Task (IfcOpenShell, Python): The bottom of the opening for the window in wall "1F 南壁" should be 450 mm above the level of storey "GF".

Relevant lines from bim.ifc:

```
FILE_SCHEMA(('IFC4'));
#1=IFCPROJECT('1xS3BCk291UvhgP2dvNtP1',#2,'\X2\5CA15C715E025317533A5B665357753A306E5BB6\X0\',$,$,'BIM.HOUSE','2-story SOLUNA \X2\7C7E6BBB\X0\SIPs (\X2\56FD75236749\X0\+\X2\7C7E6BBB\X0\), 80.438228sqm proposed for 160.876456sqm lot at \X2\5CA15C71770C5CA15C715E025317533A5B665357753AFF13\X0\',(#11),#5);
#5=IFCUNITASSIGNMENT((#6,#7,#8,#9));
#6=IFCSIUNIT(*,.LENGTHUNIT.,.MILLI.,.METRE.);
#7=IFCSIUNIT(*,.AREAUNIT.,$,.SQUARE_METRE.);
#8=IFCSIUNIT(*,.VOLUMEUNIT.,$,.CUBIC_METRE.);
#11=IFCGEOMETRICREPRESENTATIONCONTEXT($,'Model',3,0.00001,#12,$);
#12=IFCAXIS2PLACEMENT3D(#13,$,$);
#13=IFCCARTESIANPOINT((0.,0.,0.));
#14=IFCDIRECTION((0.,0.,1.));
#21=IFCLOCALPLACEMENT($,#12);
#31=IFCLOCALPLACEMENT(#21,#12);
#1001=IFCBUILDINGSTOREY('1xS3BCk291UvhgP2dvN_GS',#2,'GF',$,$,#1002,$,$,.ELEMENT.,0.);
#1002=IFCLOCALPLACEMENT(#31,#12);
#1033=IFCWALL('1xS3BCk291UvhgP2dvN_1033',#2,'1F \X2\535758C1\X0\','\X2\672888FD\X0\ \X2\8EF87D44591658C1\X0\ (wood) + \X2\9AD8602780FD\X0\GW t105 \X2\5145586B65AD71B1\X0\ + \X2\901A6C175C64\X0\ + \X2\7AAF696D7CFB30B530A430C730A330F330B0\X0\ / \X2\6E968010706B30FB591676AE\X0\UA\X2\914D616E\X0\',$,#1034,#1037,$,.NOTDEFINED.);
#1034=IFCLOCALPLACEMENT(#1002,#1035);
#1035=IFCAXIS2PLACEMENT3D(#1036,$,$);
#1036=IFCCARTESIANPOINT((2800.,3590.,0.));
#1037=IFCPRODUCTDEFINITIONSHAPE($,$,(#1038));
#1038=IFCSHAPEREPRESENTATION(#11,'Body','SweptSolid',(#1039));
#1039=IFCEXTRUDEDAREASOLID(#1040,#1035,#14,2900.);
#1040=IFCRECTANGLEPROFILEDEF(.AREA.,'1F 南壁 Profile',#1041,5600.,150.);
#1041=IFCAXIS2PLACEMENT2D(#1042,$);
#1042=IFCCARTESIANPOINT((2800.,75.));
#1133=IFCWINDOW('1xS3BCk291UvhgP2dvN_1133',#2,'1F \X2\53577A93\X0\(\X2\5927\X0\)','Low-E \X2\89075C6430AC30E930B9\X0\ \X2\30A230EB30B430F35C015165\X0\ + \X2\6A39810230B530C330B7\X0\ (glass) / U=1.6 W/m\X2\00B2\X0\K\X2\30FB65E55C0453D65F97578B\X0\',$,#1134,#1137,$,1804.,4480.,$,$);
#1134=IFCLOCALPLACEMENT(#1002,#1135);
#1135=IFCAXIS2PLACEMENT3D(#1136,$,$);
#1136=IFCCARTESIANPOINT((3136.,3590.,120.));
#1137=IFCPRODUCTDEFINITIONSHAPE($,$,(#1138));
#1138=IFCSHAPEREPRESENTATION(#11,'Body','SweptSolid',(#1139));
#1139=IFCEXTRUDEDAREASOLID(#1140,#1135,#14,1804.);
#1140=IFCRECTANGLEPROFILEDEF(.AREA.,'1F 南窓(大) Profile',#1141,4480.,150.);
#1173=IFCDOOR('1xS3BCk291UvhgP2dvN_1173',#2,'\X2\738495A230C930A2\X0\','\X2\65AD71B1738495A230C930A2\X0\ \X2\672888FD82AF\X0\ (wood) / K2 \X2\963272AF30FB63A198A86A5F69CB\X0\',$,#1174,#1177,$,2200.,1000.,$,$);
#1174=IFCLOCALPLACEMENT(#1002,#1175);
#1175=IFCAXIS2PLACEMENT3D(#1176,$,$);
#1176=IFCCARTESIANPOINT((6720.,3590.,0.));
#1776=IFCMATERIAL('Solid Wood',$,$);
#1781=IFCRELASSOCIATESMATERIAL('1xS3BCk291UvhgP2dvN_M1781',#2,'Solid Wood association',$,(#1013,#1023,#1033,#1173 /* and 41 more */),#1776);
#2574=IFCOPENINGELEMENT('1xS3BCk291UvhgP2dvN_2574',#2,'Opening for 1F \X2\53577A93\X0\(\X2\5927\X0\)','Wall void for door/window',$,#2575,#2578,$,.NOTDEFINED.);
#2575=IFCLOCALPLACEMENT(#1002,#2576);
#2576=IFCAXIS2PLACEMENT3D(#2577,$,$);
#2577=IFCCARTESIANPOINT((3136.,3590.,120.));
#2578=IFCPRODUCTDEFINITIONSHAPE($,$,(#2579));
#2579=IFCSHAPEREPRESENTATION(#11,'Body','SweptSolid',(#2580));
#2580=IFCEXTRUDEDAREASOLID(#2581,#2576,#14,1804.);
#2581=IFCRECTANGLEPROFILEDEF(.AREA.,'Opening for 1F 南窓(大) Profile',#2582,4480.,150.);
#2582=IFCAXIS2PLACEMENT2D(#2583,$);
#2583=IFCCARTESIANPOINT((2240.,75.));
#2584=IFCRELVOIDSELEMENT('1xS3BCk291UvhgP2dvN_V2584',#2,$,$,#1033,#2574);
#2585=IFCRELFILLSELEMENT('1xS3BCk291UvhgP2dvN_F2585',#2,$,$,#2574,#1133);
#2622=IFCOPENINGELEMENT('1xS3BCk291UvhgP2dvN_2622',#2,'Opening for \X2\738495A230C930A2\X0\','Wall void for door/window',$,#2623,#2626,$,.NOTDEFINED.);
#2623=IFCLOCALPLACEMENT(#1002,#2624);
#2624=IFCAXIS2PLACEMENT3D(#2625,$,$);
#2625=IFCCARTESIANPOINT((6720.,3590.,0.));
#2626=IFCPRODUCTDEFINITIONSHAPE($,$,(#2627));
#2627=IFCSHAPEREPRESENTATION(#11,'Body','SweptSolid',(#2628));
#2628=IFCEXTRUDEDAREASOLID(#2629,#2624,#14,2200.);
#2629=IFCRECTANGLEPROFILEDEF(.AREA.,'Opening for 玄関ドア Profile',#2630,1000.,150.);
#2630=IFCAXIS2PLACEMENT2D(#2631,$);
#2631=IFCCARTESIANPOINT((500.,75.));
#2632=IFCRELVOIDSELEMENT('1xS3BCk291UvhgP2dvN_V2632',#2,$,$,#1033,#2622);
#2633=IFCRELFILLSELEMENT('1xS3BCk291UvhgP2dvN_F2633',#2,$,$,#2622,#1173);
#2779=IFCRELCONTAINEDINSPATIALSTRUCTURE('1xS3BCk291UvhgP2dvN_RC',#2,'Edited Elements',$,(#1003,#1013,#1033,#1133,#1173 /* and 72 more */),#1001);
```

```python
import numpy as np
import ifcopenshell
import ifcopenshell.api.geometry
import ifcopenshell.geom
import ifcopenshell.util.element
import ifcopenshell.util.placement
import ifcopenshell.util.shape
import ifcopenshell.util.unit

model = ifcopenshell.open("bim.ifc")
unit_scale = ifcopenshell.util.unit.calculate_unit_scale(model)

window = model.by_id(1133)
opening = window.FillsVoids[0].RelatingOpeningElement
storey = ifcopenshell.util.element.get_container(window, ifc_class="IfcBuildingStorey")
level = ifcopenshell.util.placement.get_local_placement(storey.ObjectPlacement)[2, 3]

# The opening's origin need not be at the sill, so measure its lowest point.
shape = ifcopenshell.geom.create_shape(ifcopenshell.geom.settings(), opening)
bottom = ifcopenshell.util.shape.get_shape_bottom_elevation(shape, shape.geometry) / unit_scale
dz = level + 450.0 - bottom

shift = np.array([0.0, 0.0, dz])
# The window is not placed relative to its opening, so move both.
for product in (opening, window):
    matrix = ifcopenshell.util.placement.get_local_placement(product.ObjectPlacement)
    matrix[:3, 3] += shift
    ifcopenshell.api.geometry.edit_object_placement(model, product=product, matrix=matrix, is_si=False)

print(f"moved by {dz * unit_scale:+.3f} m")

model.write("bim_updated.ifc")
```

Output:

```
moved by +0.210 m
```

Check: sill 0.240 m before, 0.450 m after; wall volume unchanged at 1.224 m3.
